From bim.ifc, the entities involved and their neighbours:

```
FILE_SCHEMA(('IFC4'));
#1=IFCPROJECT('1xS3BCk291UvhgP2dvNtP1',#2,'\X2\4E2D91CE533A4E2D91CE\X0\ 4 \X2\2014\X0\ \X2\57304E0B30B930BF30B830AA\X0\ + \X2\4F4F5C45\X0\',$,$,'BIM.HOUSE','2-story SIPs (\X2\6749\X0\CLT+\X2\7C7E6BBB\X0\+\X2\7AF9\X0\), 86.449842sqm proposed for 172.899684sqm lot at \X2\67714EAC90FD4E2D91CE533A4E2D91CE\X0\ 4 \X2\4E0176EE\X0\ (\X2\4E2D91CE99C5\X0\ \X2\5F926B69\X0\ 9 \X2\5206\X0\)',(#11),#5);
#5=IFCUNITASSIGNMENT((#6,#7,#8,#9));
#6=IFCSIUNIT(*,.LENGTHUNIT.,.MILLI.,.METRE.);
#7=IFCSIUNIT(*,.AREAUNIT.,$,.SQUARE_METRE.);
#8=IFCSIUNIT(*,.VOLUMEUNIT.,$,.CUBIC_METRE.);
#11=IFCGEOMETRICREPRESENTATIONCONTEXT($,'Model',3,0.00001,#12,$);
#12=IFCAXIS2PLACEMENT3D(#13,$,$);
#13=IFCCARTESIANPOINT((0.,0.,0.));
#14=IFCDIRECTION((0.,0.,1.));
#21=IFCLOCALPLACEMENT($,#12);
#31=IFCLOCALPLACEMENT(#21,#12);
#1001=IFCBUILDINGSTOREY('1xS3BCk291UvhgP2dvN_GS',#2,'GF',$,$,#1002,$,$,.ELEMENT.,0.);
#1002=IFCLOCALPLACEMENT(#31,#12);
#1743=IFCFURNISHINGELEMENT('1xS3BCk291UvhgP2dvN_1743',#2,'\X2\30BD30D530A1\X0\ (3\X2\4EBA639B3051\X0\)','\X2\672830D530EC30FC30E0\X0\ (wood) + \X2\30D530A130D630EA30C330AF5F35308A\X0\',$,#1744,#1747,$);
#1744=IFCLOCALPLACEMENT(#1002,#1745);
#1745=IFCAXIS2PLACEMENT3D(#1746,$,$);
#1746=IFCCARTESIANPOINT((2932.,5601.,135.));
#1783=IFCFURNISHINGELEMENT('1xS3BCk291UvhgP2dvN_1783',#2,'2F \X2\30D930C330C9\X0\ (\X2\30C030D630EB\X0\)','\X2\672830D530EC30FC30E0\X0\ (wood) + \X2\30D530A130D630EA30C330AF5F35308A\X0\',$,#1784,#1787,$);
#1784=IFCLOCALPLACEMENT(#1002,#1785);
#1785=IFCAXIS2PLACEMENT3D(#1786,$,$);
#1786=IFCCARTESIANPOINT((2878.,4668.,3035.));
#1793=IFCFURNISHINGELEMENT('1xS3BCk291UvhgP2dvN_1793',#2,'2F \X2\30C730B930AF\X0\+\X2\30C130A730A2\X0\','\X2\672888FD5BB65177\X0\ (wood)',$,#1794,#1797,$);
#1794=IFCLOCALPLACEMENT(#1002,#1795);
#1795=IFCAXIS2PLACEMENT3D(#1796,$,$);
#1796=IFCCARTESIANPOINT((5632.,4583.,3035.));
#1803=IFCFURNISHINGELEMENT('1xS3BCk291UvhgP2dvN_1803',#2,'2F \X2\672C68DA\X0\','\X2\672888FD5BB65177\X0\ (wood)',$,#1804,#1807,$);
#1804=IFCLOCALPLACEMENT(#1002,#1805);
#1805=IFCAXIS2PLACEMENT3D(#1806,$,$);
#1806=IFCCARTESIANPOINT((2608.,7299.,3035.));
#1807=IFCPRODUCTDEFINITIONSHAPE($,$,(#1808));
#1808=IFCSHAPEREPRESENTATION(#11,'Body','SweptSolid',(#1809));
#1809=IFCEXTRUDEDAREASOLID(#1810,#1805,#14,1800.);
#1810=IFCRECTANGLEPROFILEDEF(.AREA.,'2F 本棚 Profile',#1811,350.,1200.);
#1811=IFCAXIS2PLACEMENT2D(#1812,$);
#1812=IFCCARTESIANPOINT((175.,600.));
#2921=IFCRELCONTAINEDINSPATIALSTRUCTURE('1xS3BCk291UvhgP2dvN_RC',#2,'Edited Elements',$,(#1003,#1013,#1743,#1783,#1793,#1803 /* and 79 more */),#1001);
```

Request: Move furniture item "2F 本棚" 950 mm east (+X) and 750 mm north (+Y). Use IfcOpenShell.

```python
import ifcopenshell
import ifcopenshell.api.geometry
import ifcopenshell.util.placement
import ifcopenshell.util.unit

model = ifcopenshell.open("bim.ifc")
unit_scale = ifcopenshell.util.unit.calculate_unit_scale(model)

item = model.by_guid("1xS3BCk291UvhgP2dvN_1803")
matrix = ifcopenshell.util.placement.get_local_placement(item.ObjectPlacement)
matrix[0, 3] += 0.95 / unit_scale
matrix[1, 3] += 0.75 / unit_scale
ifcopenshell.api.geometry.edit_object_placement(model, product=item, matrix=matrix, is_si=False)

print(ifcopenshell.util.placement.get_local_placement(item.ObjectPlacement).round(3) + 0.0)

model.write("bim_edited.ifc")
```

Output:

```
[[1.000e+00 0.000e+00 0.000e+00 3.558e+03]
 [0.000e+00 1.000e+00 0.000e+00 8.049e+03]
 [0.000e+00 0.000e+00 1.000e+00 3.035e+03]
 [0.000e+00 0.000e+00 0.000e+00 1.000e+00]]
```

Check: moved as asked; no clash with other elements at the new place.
